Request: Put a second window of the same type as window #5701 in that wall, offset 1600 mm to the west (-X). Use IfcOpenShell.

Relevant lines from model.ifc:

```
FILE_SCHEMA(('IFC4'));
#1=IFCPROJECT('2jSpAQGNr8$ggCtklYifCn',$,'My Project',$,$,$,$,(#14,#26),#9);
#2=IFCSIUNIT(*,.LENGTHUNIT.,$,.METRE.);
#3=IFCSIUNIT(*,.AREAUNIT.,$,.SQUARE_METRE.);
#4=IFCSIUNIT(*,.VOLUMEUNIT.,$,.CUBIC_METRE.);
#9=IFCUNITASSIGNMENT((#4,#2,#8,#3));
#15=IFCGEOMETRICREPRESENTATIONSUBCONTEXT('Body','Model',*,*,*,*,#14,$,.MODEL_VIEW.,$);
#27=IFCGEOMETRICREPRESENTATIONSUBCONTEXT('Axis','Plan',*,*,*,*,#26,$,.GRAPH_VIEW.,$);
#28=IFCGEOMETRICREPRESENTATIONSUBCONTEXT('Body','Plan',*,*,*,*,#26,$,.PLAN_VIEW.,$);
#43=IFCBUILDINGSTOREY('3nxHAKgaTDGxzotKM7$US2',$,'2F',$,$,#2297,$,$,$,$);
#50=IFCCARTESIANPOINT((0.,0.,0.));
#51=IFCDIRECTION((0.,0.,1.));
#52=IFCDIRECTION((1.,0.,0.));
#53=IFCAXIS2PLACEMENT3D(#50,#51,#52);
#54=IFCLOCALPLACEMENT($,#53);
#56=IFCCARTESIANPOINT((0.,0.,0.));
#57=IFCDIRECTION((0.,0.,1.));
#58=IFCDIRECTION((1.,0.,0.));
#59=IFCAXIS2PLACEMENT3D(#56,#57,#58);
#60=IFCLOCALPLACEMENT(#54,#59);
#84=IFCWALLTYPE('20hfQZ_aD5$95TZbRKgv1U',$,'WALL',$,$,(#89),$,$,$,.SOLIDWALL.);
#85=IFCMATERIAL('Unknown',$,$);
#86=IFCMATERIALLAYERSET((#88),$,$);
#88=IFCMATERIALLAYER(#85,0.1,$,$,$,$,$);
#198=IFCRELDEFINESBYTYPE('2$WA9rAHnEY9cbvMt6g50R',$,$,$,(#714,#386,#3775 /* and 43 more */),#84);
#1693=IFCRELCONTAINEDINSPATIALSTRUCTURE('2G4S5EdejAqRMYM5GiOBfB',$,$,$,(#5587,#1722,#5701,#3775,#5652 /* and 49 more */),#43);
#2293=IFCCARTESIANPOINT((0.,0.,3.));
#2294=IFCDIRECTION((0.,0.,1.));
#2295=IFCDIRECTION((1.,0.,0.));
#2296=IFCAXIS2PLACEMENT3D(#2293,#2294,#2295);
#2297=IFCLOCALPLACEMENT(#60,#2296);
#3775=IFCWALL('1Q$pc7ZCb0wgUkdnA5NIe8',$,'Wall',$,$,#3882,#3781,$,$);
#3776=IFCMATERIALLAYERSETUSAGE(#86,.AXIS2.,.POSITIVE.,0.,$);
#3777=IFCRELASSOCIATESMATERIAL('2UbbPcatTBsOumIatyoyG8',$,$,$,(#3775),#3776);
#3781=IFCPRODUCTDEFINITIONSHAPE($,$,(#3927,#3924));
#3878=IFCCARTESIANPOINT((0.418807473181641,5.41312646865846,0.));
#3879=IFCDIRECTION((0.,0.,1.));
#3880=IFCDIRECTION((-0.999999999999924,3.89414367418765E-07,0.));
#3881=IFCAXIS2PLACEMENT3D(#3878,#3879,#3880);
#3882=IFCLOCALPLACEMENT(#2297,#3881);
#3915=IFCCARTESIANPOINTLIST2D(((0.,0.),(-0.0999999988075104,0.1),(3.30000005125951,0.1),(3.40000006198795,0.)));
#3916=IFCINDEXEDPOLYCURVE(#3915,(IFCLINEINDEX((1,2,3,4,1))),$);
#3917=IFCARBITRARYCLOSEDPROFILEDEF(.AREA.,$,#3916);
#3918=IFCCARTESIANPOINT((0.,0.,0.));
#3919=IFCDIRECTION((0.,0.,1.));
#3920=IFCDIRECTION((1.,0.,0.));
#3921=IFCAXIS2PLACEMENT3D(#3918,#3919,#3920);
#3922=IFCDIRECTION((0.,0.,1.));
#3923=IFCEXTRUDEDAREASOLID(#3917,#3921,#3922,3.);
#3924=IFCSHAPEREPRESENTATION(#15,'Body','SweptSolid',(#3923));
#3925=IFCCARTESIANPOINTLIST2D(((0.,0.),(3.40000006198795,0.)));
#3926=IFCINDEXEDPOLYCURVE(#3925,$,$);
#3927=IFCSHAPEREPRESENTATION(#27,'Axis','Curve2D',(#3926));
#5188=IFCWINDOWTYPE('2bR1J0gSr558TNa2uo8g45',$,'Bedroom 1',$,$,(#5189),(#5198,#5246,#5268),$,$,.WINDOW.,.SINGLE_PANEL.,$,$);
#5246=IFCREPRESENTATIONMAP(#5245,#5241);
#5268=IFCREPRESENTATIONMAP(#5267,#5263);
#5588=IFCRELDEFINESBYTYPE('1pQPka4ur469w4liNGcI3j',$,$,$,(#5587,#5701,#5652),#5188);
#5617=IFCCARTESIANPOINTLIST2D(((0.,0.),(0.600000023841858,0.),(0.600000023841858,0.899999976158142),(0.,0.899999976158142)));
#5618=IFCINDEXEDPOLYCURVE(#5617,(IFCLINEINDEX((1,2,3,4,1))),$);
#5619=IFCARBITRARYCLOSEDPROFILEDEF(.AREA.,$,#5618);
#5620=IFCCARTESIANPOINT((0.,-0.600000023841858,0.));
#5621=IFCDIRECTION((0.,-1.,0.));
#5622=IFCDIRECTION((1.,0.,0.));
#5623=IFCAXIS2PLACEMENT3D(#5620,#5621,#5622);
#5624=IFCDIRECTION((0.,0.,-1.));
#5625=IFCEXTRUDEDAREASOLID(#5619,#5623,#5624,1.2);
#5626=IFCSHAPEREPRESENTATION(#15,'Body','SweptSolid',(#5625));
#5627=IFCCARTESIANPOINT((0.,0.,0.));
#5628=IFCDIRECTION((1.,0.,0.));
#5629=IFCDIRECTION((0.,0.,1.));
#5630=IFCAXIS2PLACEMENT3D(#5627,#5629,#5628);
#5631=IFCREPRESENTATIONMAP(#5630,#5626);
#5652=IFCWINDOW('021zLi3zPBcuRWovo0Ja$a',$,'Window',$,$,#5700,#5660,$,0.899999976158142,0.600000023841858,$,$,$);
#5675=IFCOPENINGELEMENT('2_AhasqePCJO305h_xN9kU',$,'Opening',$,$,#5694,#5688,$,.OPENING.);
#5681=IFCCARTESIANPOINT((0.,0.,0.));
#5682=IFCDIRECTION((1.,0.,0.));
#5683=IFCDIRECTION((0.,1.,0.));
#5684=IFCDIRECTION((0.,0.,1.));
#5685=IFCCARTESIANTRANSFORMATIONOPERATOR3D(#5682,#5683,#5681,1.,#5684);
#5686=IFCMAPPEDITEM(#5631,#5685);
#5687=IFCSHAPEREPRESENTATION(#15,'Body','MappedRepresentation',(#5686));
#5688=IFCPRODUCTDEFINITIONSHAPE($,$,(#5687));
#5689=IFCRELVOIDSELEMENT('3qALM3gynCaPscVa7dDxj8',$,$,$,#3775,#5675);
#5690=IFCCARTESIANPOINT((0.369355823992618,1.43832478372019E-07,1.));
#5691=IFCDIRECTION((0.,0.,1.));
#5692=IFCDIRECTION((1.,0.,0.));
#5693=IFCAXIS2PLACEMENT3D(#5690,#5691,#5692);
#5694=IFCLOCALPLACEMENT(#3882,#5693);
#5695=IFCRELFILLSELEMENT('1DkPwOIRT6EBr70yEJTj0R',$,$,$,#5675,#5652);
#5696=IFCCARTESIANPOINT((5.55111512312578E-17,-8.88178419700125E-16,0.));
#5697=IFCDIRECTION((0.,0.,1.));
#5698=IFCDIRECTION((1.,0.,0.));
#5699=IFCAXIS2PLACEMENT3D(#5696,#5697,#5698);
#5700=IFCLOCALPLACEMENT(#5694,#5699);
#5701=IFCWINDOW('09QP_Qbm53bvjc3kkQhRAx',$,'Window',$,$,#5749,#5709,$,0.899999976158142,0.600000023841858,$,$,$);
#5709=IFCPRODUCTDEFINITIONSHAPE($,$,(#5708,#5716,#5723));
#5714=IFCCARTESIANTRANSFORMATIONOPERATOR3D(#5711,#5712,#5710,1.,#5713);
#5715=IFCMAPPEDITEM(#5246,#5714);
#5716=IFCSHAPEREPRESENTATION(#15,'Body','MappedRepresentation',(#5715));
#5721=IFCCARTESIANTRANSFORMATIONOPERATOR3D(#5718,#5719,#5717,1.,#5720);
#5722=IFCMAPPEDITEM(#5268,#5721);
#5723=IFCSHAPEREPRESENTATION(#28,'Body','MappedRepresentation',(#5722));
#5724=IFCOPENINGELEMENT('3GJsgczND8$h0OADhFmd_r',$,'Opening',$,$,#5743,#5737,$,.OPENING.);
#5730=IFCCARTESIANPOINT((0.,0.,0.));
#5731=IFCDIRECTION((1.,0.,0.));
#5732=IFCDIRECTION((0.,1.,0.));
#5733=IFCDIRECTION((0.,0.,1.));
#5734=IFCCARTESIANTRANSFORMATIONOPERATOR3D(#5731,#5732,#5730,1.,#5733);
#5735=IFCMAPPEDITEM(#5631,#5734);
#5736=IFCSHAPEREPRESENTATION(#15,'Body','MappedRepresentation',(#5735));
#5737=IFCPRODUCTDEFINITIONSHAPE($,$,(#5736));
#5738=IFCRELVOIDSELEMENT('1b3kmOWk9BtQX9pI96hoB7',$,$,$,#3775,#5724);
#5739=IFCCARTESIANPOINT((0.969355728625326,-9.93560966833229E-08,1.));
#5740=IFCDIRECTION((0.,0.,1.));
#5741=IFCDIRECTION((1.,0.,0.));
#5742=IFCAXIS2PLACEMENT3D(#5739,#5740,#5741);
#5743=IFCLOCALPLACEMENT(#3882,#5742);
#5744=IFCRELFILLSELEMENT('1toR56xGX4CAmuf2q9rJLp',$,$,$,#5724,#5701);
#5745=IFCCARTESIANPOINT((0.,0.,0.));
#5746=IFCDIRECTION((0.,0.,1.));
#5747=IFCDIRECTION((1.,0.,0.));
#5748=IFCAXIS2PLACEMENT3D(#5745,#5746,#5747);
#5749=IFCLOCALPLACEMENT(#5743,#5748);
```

```python
import ifcopenshell
import ifcopenshell.api.feature
import ifcopenshell.api.geometry
import ifcopenshell.api.root
import ifcopenshell.geom
import ifcopenshell.util.element
import ifcopenshell.util.placement
import ifcopenshell.util.shape
import ifcopenshell.util.unit

model = ifcopenshell.open("model.ifc")
unit_scale = ifcopenshell.util.unit.calculate_unit_scale(model)
settings = ifcopenshell.geom.settings()


def volume(element):
    """Net volume in cubic metres, openings subtracted."""
    shape = ifcopenshell.geom.create_shape(settings, element)
    return ifcopenshell.util.shape.get_volume(shape.geometry)


window = model.by_guid("09QP_Qbm53bvjc3kkQhRAx")
opening = window.FillsVoids[0].RelatingOpeningElement
wall = opening.VoidsElements[0].RelatingBuildingElement
before = volume(wall)
shift = ifcopenshell.util.placement.get_local_placement(wall.ObjectPlacement)[:3, 0] * 1.6 / unit_scale

# copy_class copies the void relationship, type, container and properties, but no geometry.
new_opening = ifcopenshell.api.root.copy_class(model, product=opening)
new_opening.Representation = ifcopenshell.util.element.copy_deep(
    model, opening.Representation, exclude=["IfcGeometricRepresentationContext", "IfcRepresentationMap"]
)
new_window = ifcopenshell.api.root.copy_class(model, product=window)
new_window.Representation = ifcopenshell.util.element.copy_deep(
    model, window.Representation, exclude=["IfcGeometricRepresentationContext", "IfcRepresentationMap"]
)
ifcopenshell.api.feature.add_filling(model, opening=new_opening, element=new_window)

for old, new in ((opening, new_opening), (window, new_window)):
    matrix = ifcopenshell.util.placement.get_local_placement(old.ObjectPlacement)
    matrix[:3, 3] += shift
    ifcopenshell.api.geometry.edit_object_placement(model, product=new, matrix=matrix, is_si=False)

after = volume(wall)

print(f"wall volume {before:.3f} -> {after:.3f} m3")

model.write("model_edited.ifc")
```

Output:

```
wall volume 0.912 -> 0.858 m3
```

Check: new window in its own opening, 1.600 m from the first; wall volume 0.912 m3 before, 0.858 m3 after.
